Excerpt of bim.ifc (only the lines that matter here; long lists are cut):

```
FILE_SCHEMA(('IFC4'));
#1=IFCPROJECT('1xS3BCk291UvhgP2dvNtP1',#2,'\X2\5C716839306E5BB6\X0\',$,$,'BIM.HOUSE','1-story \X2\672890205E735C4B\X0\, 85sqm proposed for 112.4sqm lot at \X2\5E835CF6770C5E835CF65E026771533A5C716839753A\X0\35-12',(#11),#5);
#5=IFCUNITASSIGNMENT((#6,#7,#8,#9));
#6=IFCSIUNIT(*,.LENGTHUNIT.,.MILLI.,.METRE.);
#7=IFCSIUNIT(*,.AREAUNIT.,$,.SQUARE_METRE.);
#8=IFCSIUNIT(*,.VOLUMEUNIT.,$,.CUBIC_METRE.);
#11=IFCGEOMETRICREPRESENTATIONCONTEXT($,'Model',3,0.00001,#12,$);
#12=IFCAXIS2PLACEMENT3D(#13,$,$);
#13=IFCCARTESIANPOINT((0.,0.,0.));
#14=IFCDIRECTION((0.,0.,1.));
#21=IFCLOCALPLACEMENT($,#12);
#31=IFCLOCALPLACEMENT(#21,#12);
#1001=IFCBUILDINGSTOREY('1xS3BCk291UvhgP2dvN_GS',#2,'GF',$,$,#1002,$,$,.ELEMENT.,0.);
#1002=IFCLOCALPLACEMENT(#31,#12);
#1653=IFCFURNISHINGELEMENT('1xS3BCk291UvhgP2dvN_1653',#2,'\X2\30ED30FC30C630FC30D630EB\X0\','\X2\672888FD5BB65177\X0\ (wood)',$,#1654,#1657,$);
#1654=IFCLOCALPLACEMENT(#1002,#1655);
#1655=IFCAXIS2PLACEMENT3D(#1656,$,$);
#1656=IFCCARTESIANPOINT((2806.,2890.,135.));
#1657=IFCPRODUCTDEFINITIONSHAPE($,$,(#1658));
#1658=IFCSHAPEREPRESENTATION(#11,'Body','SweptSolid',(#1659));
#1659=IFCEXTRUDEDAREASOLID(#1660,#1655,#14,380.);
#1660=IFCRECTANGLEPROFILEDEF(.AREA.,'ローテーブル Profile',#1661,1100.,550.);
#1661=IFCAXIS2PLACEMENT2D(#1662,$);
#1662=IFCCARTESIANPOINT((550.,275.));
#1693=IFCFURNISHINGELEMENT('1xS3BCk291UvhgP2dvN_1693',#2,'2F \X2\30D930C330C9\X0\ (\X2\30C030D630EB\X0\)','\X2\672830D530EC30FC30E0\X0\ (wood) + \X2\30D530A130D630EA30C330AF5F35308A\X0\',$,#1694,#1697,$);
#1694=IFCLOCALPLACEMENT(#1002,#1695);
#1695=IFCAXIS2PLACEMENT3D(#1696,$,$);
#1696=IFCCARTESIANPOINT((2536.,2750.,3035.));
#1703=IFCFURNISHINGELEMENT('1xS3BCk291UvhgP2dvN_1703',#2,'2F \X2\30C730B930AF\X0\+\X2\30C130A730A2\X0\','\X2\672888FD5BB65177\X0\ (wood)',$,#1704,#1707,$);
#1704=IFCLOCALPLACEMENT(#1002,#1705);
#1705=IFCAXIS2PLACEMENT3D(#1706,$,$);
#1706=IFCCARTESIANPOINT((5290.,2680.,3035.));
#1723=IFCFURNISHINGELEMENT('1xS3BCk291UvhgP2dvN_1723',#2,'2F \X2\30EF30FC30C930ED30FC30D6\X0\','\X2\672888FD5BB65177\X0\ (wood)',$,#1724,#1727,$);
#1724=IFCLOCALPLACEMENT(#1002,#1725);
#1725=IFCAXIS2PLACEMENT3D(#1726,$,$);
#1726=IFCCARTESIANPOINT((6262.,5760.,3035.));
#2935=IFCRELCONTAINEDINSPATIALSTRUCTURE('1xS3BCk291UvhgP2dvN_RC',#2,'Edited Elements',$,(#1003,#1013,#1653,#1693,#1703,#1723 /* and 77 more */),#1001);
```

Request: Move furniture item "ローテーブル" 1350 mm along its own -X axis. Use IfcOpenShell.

```python
import ifcopenshell
import ifcopenshell.api.geometry
import ifcopenshell.util.placement
import ifcopenshell.util.unit

model = ifcopenshell.open("bim.ifc")
unit_scale = ifcopenshell.util.unit.calculate_unit_scale(model)

item = model.by_id(1653)
matrix = ifcopenshell.util.placement.get_local_placement(item.ObjectPlacement)
matrix[:3, 3] -= matrix[:3, 0] * 1.35 / unit_scale
ifcopenshell.api.geometry.edit_object_placement(model, product=item, matrix=matrix, is_si=False)

print(ifcopenshell.util.placement.get_local_placement(item.ObjectPlacement).round(3) + 0.0)

model.write("bim_v2.ifc")
```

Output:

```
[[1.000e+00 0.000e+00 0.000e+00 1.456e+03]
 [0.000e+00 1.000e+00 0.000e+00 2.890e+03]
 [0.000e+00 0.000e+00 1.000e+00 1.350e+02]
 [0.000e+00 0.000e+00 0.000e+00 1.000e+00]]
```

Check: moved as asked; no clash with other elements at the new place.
